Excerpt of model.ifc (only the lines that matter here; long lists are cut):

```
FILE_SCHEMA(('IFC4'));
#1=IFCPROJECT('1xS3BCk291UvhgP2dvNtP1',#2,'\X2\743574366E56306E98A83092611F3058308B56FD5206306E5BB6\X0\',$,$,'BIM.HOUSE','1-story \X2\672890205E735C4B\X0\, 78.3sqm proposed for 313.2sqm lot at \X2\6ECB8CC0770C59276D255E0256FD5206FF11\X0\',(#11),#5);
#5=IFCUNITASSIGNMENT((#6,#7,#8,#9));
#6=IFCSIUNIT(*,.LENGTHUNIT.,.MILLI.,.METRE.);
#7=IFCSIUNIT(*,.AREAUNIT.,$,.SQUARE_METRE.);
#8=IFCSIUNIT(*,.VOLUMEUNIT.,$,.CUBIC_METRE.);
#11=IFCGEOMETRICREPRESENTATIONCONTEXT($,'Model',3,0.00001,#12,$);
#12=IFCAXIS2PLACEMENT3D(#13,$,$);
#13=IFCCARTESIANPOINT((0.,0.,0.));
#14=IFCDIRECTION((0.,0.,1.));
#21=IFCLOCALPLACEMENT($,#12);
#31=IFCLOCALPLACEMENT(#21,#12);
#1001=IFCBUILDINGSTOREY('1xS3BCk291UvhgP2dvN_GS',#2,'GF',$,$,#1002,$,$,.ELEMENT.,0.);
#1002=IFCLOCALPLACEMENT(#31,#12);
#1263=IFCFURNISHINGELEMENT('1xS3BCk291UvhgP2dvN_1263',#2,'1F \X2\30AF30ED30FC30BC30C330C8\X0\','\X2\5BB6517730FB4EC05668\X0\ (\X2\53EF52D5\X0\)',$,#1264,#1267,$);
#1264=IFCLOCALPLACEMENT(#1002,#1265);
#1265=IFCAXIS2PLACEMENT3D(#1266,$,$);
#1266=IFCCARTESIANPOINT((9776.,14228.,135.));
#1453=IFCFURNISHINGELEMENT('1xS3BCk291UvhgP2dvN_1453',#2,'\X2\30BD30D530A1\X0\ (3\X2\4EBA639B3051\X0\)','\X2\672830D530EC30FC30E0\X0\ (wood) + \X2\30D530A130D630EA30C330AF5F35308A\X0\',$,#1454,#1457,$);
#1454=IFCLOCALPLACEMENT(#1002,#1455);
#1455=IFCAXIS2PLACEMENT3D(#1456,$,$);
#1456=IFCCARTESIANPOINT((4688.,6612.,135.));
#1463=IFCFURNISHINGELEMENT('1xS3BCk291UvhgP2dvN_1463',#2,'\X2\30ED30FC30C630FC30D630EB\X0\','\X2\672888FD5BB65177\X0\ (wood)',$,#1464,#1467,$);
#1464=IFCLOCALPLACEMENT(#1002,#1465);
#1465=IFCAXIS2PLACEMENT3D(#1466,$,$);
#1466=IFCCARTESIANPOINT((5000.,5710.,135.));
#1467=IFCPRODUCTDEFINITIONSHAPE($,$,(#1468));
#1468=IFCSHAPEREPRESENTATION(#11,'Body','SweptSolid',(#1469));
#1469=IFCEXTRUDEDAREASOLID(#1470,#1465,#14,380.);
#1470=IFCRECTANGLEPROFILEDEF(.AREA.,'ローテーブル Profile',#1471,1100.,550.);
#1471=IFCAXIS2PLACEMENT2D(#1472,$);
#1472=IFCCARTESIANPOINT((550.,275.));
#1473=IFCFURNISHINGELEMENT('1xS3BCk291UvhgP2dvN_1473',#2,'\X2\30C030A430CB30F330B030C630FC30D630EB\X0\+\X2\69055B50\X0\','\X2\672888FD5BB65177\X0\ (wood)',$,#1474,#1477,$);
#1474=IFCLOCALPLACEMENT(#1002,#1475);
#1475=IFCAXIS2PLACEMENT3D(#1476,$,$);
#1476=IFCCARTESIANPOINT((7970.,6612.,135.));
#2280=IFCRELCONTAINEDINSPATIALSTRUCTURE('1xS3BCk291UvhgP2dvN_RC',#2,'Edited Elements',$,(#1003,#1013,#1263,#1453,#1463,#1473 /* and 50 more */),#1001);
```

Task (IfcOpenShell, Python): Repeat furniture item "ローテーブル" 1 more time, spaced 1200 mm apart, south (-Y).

```python
import numpy as np
import ifcopenshell
import ifcopenshell.api.geometry
import ifcopenshell.api.root
import ifcopenshell.util.element
import ifcopenshell.util.placement
import ifcopenshell.util.unit

model = ifcopenshell.open("model.ifc")
unit_scale = ifcopenshell.util.unit.calculate_unit_scale(model)


def reuse_history(source, copy):
    """copy_class also copies each property set's owner history, people and application; keep the originals."""
    for rel in copy.IsDefinedBy:
        if rel.is_a("IfcRelDefinesByProperties") and (history := rel.RelatingPropertyDefinition.OwnerHistory):
            rel.RelatingPropertyDefinition.OwnerHistory = source.OwnerHistory
            ifcopenshell.util.element.remove_deep2(model, history)


source = model.by_id(1463)
base = ifcopenshell.util.placement.get_local_placement(source.ObjectPlacement)
step = np.array([0.0, -1.0, 0.0]) * 1.2 / unit_scale

for i in range(1, 2):
    copy = ifcopenshell.api.root.copy_class(model, product=source)
    copy.Representation = ifcopenshell.util.element.copy_deep(
        model, source.Representation, exclude=["IfcGeometricRepresentationContext", "IfcRepresentationMap"]
    )
    reuse_history(source, copy)
    matrix = base.copy()
    matrix[:3, 3] += i * step
    print("added at", matrix[:3, 3].round(3) + 0.0)
    ifcopenshell.api.geometry.edit_object_placement(model, product=copy, matrix=matrix, is_si=False)

model.write("model_rev.ifc")
```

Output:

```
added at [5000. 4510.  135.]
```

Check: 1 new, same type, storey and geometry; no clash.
